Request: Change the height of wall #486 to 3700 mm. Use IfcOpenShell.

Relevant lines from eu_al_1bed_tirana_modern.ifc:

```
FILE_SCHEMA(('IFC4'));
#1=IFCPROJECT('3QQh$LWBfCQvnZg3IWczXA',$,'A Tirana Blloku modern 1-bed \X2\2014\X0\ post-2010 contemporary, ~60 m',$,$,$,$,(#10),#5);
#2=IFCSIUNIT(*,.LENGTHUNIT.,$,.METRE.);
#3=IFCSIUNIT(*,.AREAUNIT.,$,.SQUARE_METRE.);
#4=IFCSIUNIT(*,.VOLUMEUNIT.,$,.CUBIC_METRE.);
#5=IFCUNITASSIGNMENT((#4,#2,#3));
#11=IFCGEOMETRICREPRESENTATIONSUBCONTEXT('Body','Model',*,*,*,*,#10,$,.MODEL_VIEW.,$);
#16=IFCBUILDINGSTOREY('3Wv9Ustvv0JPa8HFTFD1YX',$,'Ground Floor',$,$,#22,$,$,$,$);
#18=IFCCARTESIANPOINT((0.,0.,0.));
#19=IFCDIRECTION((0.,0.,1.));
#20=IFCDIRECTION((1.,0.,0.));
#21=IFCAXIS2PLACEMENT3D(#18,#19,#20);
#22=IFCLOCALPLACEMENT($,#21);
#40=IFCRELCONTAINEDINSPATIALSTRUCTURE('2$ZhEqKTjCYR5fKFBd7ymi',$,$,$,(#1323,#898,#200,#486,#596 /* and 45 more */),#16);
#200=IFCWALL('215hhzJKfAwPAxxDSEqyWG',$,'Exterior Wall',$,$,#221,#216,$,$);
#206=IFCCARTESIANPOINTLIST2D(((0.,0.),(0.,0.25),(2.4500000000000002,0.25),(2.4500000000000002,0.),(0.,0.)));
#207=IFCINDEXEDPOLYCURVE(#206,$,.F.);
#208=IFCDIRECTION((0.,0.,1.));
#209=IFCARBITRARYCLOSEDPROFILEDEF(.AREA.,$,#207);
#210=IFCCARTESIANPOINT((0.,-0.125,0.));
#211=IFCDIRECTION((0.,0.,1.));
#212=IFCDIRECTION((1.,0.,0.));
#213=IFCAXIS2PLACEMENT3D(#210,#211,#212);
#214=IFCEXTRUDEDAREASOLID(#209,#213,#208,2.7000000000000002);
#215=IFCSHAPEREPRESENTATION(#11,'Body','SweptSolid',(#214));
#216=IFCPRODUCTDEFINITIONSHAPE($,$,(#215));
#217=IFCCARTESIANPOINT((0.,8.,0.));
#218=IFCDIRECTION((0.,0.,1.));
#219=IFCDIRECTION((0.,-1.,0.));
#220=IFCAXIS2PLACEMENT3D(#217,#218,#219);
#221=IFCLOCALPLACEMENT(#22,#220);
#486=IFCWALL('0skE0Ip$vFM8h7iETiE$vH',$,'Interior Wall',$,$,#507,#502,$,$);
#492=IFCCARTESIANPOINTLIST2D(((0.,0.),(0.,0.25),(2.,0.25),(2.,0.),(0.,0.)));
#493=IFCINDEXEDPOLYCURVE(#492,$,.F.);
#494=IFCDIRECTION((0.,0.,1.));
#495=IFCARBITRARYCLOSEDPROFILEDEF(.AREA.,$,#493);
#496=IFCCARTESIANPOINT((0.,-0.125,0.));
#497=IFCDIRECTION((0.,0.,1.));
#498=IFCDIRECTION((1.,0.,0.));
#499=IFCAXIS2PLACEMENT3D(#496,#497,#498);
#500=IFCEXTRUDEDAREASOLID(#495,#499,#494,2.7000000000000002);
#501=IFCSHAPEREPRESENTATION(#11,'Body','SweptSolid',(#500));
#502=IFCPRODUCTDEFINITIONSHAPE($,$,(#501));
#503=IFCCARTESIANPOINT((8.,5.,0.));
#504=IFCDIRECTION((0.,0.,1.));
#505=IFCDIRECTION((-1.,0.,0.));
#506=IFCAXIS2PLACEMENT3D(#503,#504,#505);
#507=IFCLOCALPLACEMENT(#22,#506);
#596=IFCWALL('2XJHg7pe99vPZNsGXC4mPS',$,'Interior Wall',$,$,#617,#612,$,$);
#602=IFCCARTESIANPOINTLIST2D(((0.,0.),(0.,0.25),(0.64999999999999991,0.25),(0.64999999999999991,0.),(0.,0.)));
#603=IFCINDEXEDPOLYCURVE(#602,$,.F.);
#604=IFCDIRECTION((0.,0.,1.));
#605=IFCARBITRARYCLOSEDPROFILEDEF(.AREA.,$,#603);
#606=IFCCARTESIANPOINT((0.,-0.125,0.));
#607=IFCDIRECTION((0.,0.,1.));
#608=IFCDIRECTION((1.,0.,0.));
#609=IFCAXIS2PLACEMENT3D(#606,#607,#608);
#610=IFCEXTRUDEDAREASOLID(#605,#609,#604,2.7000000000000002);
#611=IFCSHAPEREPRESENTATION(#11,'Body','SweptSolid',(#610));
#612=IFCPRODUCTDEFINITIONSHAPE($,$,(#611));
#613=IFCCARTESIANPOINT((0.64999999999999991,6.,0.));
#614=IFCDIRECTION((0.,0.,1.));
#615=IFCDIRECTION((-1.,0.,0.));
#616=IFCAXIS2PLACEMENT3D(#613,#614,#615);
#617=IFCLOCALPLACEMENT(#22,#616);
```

```python
import ifcopenshell
import ifcopenshell.geom
import ifcopenshell.util.representation
import ifcopenshell.util.shape
import ifcopenshell.util.unit

model = ifcopenshell.open("eu_al_1bed_tirana_modern.ifc")
unit_scale = ifcopenshell.util.unit.calculate_unit_scale(model)
settings = ifcopenshell.geom.settings()


def volume(element):
    """Net volume in cubic metres, openings subtracted."""
    shape = ifcopenshell.geom.create_shape(settings, element)
    return ifcopenshell.util.shape.get_volume(shape.geometry)


wall = model.by_id(486)
before = volume(wall)

body = ifcopenshell.util.representation.get_representation(wall, "Model", "Body")
solid = body.Items[0]
old_height = solid.Depth
solid.Depth = 3.7 / unit_scale
after = volume(wall)

print(f"height {old_height:g} -> {solid.Depth:g}, volume {before:.3f} -> {after:.3f} m3")

model.write("eu_al_1bed_tirana_modern_edited.ifc")
```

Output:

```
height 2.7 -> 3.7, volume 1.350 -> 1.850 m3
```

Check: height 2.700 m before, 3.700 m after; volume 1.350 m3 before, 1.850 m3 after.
